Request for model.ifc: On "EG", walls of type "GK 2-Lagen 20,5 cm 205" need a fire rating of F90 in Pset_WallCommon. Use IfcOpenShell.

First a look at what the model holds.

```python
import ifcopenshell
import ifcopenshell.util.element

model = ifcopenshell.open("model.ifc")
print(model.schema)
storey = next(s for s in model.by_type("IfcBuildingStorey") if s.Name == "EG")
walls = [e for e in ifcopenshell.util.element.get_decomposition(storey) if e.is_a("IfcWall")]
seen = {}
for e in walls:
    element_type = ifcopenshell.util.element.get_type(e)
    key = (element_type.Name if element_type != e and element_type else None, ifcopenshell.util.element.get_pset(e, "Pset_WallCommon", "FireRating"))
    seen[key] = seen.get(key, 0) + 1
for (name, value), count in sorted(seen.items(), key=str):
    print(count, "x", name, "|", value)
```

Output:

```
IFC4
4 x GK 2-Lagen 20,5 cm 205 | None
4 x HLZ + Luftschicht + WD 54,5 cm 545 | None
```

```python
import ifcopenshell
import ifcopenshell.api.pset
import ifcopenshell.util.element

model = ifcopenshell.open("model.ifc")

storey = next(s for s in model.by_type("IfcBuildingStorey") if s.Name == "EG")
walls = [e for e in ifcopenshell.util.element.get_decomposition(storey) if e.is_a("IfcWall")]

count = 0
for e in walls:
    element_type = ifcopenshell.util.element.get_type(e)
    if element_type in (None, e) or element_type.Name != "GK 2-Lagen 20,5 cm 205":
        continue
    # add_pset returns the element's existing set when there is one.
    pset = ifcopenshell.api.pset.add_pset(model, product=e, name="Pset_WallCommon")
    ifcopenshell.api.pset.edit_pset(model, pset=pset, properties={"FireRating": "F90"})
    count += 1

print(count, "walls updated")

model.write("model_edited.ifc")
```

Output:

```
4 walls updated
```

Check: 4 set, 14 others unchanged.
